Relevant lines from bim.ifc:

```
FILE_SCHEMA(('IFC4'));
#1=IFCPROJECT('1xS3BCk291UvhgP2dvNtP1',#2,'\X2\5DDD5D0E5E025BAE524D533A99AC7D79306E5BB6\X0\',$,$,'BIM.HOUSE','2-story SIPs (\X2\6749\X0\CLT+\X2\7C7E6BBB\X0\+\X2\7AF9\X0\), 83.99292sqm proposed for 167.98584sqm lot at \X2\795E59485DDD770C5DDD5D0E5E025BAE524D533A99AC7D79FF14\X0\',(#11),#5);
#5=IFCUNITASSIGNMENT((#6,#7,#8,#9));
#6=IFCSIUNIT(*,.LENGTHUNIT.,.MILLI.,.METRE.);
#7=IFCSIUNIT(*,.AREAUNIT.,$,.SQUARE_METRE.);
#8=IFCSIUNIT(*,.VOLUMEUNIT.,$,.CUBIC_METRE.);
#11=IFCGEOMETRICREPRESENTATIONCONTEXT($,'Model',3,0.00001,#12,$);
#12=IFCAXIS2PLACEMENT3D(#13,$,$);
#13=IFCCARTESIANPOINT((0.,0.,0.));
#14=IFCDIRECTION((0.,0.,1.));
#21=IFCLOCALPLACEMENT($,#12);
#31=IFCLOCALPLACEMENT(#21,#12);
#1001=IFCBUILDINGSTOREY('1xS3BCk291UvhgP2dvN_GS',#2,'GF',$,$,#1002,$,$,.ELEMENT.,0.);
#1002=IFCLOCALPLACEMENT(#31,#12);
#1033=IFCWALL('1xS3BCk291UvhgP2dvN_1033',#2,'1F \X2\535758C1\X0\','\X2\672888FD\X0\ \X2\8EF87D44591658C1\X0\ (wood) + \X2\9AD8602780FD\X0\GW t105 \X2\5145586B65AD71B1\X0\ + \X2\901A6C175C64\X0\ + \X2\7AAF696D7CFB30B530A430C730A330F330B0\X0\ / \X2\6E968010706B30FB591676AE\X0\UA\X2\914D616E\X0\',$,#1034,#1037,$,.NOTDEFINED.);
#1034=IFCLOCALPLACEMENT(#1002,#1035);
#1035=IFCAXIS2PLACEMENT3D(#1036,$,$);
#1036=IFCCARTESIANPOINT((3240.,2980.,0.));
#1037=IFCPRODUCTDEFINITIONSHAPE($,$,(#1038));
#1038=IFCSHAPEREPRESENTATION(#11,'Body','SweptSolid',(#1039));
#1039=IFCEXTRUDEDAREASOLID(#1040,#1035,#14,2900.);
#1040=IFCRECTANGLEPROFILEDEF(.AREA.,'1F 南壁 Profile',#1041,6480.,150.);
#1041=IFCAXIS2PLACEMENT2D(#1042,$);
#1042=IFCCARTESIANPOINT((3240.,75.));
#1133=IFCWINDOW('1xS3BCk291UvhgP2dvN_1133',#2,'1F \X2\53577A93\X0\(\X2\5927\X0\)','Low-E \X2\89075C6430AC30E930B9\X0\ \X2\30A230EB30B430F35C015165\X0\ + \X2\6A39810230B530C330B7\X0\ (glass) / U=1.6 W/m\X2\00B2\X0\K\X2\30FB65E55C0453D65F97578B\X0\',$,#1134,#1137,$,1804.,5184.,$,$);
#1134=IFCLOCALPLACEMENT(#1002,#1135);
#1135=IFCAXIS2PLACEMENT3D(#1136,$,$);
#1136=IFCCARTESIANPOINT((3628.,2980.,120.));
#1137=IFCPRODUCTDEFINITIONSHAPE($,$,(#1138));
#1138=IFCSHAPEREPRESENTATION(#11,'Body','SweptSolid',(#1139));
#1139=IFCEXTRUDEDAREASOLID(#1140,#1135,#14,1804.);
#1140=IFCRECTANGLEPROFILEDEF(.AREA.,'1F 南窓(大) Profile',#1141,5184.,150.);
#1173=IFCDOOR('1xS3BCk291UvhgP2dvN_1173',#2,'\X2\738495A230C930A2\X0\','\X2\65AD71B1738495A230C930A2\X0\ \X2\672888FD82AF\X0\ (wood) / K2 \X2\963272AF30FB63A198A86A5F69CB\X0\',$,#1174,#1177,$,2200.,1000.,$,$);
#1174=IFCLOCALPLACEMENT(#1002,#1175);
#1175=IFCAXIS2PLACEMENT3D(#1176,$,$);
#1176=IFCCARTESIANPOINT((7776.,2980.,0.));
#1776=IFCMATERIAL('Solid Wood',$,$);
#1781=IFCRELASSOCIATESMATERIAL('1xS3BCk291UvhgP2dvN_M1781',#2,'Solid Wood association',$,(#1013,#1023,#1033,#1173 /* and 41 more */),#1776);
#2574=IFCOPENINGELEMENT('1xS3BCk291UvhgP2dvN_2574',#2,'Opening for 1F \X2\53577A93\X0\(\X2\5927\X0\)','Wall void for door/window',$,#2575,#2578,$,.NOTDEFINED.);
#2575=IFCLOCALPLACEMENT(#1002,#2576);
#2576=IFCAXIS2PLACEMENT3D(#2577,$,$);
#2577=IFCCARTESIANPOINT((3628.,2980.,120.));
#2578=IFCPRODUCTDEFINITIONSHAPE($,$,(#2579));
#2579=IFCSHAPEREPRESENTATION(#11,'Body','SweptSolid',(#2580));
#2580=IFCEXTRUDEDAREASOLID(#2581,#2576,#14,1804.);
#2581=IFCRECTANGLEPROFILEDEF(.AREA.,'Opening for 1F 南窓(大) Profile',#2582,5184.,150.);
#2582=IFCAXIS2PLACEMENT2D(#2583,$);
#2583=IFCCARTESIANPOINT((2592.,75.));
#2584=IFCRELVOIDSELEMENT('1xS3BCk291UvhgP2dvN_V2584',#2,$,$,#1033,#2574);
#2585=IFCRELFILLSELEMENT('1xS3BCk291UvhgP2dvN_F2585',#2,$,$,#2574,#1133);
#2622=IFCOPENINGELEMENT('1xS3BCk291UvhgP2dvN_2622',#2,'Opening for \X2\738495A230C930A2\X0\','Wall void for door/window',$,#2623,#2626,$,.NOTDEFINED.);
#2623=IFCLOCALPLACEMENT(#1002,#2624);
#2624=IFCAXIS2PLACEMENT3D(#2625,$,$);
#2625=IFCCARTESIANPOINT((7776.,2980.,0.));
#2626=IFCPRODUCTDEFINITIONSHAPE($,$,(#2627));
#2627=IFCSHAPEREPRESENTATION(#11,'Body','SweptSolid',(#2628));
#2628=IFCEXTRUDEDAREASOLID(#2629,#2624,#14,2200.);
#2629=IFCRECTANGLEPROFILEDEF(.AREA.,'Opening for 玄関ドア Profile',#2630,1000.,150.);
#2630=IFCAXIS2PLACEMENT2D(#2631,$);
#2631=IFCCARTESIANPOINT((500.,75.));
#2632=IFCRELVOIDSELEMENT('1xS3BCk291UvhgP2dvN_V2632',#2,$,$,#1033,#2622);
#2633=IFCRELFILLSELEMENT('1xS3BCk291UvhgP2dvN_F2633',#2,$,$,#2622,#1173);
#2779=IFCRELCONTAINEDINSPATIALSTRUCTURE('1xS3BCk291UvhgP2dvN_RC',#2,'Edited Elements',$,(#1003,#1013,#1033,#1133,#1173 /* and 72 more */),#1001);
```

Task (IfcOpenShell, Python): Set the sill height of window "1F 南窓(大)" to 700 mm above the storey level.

```python
import numpy as np
import ifcopenshell
import ifcopenshell.api.geometry
import ifcopenshell.geom
import ifcopenshell.util.element
import ifcopenshell.util.placement
import ifcopenshell.util.shape
import ifcopenshell.util.unit

model = ifcopenshell.open("bim.ifc")
unit_scale = ifcopenshell.util.unit.calculate_unit_scale(model)

window = model.by_guid("1xS3BCk291UvhgP2dvN_1133")
opening = window.FillsVoids[0].RelatingOpeningElement
storey = ifcopenshell.util.element.get_container(window, ifc_class="IfcBuildingStorey")
level = ifcopenshell.util.placement.get_local_placement(storey.ObjectPlacement)[2, 3]

# The opening's origin need not be at the sill, so measure its lowest point.
shape = ifcopenshell.geom.create_shape(ifcopenshell.geom.settings(), opening)
bottom = ifcopenshell.util.shape.get_shape_bottom_elevation(shape, shape.geometry) / unit_scale
dz = level + 0.7 / unit_scale - bottom

shift = np.array([0.0, 0.0, dz])
# The window is not placed relative to its opening, so move both.
for product in (opening, window):
    matrix = ifcopenshell.util.placement.get_local_placement(product.ObjectPlacement)
    matrix[:3, 3] += shift
    ifcopenshell.api.geometry.edit_object_placement(model, product=product, matrix=matrix, is_si=False)

print(f"moved by {dz * unit_scale:+.3f} m")

model.write("bim_updated.ifc")
```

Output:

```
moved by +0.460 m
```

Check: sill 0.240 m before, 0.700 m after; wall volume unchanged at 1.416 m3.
